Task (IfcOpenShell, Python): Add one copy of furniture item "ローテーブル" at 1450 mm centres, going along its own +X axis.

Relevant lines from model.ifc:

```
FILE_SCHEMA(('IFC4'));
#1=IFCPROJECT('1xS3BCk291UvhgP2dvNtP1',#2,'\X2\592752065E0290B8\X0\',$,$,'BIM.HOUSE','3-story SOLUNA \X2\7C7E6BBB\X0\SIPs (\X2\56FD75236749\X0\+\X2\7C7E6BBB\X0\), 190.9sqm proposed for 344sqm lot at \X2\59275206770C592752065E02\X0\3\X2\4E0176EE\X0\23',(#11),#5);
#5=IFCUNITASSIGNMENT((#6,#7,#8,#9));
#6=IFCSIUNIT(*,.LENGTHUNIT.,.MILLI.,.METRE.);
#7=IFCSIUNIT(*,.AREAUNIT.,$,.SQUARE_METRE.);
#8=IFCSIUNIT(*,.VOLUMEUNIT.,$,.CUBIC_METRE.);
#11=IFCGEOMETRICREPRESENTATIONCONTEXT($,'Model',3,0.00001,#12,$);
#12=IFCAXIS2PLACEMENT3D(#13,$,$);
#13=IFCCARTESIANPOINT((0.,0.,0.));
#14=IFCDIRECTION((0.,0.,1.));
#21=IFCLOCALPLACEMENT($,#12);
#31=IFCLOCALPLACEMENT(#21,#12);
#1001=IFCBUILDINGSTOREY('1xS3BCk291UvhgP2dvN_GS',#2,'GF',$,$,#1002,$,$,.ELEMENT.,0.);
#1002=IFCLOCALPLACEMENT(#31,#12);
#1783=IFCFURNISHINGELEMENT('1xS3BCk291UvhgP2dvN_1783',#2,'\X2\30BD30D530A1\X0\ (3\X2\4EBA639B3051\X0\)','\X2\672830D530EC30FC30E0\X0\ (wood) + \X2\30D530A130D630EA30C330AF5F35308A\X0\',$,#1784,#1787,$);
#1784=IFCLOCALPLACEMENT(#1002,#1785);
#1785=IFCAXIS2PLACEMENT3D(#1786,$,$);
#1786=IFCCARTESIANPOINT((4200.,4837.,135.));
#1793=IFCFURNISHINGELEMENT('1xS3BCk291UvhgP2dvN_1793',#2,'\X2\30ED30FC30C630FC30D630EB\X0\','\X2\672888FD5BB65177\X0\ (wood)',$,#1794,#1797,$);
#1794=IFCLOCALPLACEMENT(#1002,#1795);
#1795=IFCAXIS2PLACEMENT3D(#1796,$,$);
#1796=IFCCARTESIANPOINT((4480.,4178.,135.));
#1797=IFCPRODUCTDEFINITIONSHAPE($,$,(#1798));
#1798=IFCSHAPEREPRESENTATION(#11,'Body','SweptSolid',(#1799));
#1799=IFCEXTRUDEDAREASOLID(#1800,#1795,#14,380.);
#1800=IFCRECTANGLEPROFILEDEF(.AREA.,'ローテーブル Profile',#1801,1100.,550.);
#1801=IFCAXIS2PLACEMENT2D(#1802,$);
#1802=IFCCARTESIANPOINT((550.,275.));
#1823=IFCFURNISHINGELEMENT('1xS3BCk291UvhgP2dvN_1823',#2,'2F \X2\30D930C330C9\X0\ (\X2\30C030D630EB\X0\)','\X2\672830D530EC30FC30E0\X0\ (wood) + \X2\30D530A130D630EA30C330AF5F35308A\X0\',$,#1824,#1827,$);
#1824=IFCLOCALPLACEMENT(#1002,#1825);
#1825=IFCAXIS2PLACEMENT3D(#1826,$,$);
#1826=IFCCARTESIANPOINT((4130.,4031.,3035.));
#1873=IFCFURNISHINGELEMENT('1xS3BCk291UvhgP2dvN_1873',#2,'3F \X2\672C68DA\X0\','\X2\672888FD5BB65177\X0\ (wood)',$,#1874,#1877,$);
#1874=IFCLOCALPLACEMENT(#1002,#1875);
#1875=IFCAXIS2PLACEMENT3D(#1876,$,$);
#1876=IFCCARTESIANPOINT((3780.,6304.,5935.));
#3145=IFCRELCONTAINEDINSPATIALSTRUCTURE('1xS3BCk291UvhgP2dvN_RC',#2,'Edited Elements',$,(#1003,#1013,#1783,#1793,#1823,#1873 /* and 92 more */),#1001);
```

```python
import ifcopenshell
import ifcopenshell.api.geometry
import ifcopenshell.api.root
import ifcopenshell.util.element
import ifcopenshell.util.placement
import ifcopenshell.util.unit

model = ifcopenshell.open("model.ifc")
unit_scale = ifcopenshell.util.unit.calculate_unit_scale(model)


def reuse_history(source, copy):
    """copy_class also copies each property set's owner history, people and application; keep the originals."""
    for rel in copy.IsDefinedBy:
        if rel.is_a("IfcRelDefinesByProperties") and (history := rel.RelatingPropertyDefinition.OwnerHistory):
            rel.RelatingPropertyDefinition.OwnerHistory = source.OwnerHistory
            ifcopenshell.util.element.remove_deep2(model, history)


source = model.by_guid("1xS3BCk291UvhgP2dvN_1793")
base = ifcopenshell.util.placement.get_local_placement(source.ObjectPlacement)
step = base[:3, 0] * 1.45 / unit_scale

for i in range(1, 2):
    copy = ifcopenshell.api.root.copy_class(model, product=source)
    copy.Representation = ifcopenshell.util.element.copy_deep(
        model, source.Representation, exclude=["IfcGeometricRepresentationContext", "IfcRepresentationMap"]
    )
    reuse_history(source, copy)
    matrix = base.copy()
    matrix[:3, 3] += i * step
    print("added at", matrix[:3, 3].round(3) + 0.0)
    ifcopenshell.api.geometry.edit_object_placement(model, product=copy, matrix=matrix, is_si=False)

model.write("model_updated.ifc")
```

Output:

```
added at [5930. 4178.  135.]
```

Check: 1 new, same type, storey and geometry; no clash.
